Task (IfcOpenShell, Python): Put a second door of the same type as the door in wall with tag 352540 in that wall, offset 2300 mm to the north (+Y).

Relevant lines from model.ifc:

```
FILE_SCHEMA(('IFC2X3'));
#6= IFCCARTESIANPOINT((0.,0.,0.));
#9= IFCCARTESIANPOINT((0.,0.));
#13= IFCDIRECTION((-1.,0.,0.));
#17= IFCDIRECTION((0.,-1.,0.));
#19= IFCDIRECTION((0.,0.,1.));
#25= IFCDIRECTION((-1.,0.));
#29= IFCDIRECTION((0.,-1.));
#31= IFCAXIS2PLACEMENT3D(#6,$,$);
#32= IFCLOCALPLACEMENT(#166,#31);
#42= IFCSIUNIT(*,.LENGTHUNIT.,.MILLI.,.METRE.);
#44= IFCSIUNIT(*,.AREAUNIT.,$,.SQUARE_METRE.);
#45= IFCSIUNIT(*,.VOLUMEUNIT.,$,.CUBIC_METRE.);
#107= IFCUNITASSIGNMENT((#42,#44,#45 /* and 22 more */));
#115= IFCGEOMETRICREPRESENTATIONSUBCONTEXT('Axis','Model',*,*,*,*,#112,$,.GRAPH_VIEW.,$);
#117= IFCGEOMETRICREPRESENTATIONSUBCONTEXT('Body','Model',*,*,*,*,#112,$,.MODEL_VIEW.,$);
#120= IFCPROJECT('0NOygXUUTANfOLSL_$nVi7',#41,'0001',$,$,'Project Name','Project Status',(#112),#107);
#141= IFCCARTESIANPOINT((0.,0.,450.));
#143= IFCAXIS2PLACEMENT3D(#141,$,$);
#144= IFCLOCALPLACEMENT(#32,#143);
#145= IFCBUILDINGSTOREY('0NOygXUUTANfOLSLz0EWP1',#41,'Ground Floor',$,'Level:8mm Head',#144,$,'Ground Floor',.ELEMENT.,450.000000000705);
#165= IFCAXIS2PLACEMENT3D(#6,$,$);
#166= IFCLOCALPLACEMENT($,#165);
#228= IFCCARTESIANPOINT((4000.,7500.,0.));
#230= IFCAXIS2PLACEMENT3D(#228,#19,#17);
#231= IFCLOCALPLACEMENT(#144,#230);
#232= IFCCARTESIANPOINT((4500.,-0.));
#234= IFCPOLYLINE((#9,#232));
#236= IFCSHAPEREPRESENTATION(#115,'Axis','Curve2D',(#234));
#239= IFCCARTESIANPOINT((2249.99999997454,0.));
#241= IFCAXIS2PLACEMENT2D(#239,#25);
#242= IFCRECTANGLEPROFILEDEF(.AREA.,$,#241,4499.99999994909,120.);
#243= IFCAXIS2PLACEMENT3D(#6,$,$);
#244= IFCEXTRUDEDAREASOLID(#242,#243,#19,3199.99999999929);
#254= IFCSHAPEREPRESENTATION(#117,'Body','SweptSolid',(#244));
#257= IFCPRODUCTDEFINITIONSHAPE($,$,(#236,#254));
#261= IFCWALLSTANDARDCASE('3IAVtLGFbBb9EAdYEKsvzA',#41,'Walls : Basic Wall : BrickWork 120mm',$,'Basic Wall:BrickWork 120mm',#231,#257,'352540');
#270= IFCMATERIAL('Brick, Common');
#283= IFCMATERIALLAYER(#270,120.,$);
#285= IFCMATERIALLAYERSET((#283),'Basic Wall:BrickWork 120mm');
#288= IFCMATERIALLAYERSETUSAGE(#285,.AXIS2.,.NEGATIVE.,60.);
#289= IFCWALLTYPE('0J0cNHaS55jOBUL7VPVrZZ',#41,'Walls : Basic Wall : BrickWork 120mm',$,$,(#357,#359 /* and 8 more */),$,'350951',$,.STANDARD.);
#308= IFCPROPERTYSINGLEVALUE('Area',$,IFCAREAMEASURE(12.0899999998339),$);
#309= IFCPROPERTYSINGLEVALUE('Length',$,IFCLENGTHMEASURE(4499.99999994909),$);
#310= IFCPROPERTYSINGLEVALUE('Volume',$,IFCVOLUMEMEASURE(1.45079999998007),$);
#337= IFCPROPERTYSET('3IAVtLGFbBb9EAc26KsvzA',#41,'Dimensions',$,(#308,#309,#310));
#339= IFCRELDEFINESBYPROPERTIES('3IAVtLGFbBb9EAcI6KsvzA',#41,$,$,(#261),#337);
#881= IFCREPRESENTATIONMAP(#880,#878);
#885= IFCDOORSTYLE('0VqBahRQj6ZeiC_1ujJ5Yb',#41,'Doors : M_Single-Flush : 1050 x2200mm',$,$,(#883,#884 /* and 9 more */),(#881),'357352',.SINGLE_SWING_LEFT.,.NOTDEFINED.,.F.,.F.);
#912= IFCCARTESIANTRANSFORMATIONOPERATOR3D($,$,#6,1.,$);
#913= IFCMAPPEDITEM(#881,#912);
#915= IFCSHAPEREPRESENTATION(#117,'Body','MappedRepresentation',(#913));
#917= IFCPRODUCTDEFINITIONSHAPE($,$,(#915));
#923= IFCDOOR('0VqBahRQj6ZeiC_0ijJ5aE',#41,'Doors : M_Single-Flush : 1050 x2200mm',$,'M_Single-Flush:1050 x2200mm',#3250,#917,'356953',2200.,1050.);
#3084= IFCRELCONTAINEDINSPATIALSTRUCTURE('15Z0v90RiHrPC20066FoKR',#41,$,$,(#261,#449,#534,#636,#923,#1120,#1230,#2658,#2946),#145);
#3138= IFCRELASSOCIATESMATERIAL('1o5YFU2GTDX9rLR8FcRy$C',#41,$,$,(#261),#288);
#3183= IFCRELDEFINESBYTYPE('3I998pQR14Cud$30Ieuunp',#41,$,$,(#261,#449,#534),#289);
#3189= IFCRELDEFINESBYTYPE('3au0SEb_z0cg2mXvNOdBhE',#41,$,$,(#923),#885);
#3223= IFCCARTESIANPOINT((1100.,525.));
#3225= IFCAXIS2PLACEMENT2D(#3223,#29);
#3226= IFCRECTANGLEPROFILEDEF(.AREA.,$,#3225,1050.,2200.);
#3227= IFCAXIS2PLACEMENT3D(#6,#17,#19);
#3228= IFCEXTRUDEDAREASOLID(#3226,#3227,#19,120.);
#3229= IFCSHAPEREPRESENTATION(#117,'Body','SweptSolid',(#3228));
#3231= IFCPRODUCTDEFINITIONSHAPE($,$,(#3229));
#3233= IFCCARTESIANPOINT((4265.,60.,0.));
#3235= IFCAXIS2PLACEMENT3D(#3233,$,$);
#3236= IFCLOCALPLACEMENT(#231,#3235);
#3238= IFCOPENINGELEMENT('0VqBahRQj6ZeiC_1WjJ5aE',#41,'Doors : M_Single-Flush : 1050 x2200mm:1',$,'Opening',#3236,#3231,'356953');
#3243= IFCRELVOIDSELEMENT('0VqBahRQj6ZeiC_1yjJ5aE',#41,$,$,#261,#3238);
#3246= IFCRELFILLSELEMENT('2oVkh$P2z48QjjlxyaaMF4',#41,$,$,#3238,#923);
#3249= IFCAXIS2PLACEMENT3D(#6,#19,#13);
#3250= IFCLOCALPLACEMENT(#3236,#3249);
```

```python
import ifcopenshell
import ifcopenshell.api.feature
import ifcopenshell.api.geometry
import ifcopenshell.api.pset
import ifcopenshell.api.root
import ifcopenshell.geom
import ifcopenshell.util.element
import ifcopenshell.util.placement
import ifcopenshell.util.shape
import ifcopenshell.util.unit

model = ifcopenshell.open("model.ifc")
unit_scale = ifcopenshell.util.unit.calculate_unit_scale(model)
area_scale = ifcopenshell.util.unit.calculate_unit_scale(model, "AREAUNIT")
volume_scale = ifcopenshell.util.unit.calculate_unit_scale(model, "VOLUMEUNIT")
settings = ifcopenshell.geom.settings()


def volume(element):
    """Net volume in cubic metres, openings subtracted."""
    shape = ifcopenshell.geom.create_shape(settings, element)
    return ifcopenshell.util.shape.get_volume(shape.geometry)


def reuse_history(source, copy):
    """copy_class also copies each property set's owner history, people and application; keep the originals."""
    for rel in copy.IsDefinedBy:
        if rel.is_a("IfcRelDefinesByProperties") and (history := rel.RelatingPropertyDefinition.OwnerHistory):
            rel.RelatingPropertyDefinition.OwnerHistory = source.OwnerHistory
            ifcopenshell.util.element.remove_deep2(model, history)


door = model.by_guid("0VqBahRQj6ZeiC_0ijJ5aE")
opening = door.FillsVoids[0].RelatingOpeningElement
wall = opening.VoidsElements[0].RelatingBuildingElement
before = volume(wall)
shift = ifcopenshell.util.placement.get_local_placement(wall.ObjectPlacement)[:3, 0] * -2.3 / unit_scale

# copy_class copies the void relationship, type, container and properties, but no geometry.
new_opening = ifcopenshell.api.root.copy_class(model, product=opening)
new_opening.Representation = ifcopenshell.util.element.copy_deep(
    model, opening.Representation, exclude=["IfcGeometricRepresentationContext", "IfcRepresentationMap"]
)
new_opening.Tag = None
new_door = ifcopenshell.api.root.copy_class(model, product=door)
new_door.Representation = ifcopenshell.util.element.copy_deep(
    model, door.Representation, exclude=["IfcGeometricRepresentationContext", "IfcRepresentationMap"]
)
new_door.Tag = None
reuse_history(door, new_door)
fills = ifcopenshell.api.feature.add_filling(model, opening=new_opening, element=new_door)
fills.OwnerHistory = new_door.OwnerHistory  # required in IFC2X3

for old, new in ((opening, new_opening), (door, new_door)):
    matrix = ifcopenshell.util.placement.get_local_placement(old.ObjectPlacement)
    matrix[:3, 3] += shift
    ifcopenshell.api.geometry.edit_object_placement(model, product=new, matrix=matrix, is_si=False)

after = volume(wall)
thickness = 0.12  # wall thickness in metres

# Update the wall's stored quantities.
pset = model.by_id(ifcopenshell.util.element.get_pset(wall, "Dimensions", should_inherit=False)["id"])
ifcopenshell.api.pset.edit_pset(model, pset=pset, properties={
    "Area": model.create_entity("IfcAreaMeasure", after / thickness / area_scale),
    "Volume": model.create_entity("IfcVolumeMeasure", after / volume_scale),
})

print(f"wall volume {before:.3f} -> {after:.3f} m3")

model.write("model_updated.ifc")
```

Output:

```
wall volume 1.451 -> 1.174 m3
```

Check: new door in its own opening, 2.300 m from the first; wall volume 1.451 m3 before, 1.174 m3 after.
